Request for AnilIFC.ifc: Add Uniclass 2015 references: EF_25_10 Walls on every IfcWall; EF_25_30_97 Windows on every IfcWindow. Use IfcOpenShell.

First a look at what the model holds.

```python
import ifcopenshell

model = ifcopenshell.open("AnilIFC.ifc")
print(model.schema)
print("classifications:", [c.Name for c in model.by_type("IfcClassification")])
for ifc_class in ("IfcDoor", "IfcRoof", "IfcStair", "IfcWall", "IfcWindow"):
    print(ifc_class, len(model.by_type(ifc_class)))
```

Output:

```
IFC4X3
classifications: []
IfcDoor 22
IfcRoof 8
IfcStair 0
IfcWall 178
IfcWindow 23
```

```python
import ifcopenshell
import ifcopenshell.api.classification

model = ifcopenshell.open("AnilIFC.ifc")

system = ifcopenshell.api.classification.add_classification(model, classification="Uniclass 2015")

codes = {
    "IfcWall": ("EF_25_10", "Walls"),
    "IfcWindow": ("EF_25_30_97", "Windows"),
}
for ifc_class, (code, name) in codes.items():
    products = model.by_type(ifc_class)
    ifcopenshell.api.classification.add_reference(
        model, products=products, classification=system, identification=code, name=name
    )
    print(code, len(products))

model.write("AnilIFC_rev.ifc")
```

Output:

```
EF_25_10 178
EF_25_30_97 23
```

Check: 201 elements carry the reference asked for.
